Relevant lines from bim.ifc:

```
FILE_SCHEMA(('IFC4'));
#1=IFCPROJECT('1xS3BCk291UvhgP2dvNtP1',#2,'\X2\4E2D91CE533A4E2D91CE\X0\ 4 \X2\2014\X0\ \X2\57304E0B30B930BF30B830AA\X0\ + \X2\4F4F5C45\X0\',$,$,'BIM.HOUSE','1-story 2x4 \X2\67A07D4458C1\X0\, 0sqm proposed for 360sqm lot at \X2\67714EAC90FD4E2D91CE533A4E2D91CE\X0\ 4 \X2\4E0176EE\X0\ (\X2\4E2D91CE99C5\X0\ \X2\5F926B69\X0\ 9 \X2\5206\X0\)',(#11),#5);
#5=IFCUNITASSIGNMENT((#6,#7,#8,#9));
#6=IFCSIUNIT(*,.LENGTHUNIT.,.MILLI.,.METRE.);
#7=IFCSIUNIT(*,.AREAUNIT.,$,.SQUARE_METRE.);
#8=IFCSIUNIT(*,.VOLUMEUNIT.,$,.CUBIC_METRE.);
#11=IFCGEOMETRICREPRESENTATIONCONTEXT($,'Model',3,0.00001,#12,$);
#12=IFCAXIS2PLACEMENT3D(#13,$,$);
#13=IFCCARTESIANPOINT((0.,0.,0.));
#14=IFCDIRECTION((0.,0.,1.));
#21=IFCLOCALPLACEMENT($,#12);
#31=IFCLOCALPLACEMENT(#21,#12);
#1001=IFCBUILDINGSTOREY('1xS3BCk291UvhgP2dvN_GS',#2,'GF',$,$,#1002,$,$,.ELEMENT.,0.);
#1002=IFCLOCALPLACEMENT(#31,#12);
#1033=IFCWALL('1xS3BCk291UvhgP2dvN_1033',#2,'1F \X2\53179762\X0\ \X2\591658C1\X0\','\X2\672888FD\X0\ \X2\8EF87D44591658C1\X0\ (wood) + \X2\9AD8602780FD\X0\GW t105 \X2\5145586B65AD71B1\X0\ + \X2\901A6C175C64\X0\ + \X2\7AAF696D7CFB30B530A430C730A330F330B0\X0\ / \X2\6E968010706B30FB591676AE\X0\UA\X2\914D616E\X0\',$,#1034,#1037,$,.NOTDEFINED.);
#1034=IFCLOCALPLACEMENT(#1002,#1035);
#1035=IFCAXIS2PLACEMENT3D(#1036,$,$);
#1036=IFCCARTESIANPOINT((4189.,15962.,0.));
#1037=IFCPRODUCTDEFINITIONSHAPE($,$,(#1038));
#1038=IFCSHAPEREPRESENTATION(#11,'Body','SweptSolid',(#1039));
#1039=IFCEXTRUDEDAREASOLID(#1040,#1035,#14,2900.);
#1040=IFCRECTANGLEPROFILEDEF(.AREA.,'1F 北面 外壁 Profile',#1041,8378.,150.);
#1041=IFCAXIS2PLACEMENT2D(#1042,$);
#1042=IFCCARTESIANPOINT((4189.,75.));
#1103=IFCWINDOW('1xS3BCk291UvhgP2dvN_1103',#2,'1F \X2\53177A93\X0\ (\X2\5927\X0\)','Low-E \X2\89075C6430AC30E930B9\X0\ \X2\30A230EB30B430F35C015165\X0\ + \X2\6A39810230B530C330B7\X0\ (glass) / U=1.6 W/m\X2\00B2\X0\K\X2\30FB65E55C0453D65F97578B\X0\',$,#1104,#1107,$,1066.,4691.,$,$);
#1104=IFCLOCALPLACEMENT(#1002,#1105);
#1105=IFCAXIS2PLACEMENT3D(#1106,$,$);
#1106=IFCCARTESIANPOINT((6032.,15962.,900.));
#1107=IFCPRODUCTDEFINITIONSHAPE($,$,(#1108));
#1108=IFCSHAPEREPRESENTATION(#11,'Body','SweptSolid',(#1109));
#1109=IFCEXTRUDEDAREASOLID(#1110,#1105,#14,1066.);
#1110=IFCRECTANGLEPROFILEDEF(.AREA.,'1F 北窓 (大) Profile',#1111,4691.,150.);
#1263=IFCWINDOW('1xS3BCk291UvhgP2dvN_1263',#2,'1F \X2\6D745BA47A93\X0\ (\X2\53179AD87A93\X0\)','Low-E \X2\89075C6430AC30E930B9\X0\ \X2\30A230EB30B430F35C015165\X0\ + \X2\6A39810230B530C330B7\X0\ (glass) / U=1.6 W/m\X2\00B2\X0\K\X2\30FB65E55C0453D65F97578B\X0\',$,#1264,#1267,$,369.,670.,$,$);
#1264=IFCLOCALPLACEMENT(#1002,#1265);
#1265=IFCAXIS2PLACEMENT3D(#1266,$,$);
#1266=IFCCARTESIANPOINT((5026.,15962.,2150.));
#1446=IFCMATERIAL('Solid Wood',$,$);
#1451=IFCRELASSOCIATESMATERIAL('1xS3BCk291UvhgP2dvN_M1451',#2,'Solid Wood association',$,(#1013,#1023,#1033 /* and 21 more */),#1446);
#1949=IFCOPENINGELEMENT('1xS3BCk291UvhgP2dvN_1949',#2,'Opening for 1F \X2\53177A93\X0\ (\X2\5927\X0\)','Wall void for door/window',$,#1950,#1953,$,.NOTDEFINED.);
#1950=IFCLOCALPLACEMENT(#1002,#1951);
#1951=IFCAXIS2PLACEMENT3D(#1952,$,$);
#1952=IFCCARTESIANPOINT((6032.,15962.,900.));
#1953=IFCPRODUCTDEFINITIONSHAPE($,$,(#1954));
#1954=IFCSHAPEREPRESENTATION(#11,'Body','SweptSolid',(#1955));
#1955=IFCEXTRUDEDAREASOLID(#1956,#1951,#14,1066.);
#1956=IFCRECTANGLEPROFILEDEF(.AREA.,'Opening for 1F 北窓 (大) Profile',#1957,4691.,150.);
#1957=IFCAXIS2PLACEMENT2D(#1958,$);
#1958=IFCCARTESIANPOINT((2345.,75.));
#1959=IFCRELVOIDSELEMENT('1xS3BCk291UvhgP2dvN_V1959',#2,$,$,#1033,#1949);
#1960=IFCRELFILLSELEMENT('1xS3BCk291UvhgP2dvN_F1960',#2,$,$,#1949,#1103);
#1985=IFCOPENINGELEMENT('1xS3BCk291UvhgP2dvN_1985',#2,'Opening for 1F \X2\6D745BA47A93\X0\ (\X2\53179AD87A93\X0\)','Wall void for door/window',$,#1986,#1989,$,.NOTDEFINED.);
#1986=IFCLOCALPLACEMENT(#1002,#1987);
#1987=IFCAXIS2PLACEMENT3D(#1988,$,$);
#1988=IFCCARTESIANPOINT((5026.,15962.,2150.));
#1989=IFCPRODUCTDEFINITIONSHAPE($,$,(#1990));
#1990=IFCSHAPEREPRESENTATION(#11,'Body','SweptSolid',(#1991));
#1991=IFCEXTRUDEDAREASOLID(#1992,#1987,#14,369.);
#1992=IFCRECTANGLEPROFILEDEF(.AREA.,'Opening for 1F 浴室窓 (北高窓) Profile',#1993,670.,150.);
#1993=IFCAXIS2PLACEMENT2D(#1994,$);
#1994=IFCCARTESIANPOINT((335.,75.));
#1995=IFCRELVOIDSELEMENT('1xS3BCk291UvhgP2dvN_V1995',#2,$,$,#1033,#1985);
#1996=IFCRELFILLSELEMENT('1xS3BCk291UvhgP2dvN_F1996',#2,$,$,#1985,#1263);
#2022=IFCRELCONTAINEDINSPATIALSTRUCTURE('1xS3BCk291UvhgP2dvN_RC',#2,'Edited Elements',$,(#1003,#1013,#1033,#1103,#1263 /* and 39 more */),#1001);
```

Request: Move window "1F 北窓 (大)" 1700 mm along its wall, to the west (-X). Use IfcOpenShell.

```python
import ifcopenshell
import ifcopenshell.api.geometry
import ifcopenshell.util.placement
import ifcopenshell.util.unit

model = ifcopenshell.open("bim.ifc")
unit_scale = ifcopenshell.util.unit.calculate_unit_scale(model)

window = model.by_id(1103)
opening = window.FillsVoids[0].RelatingOpeningElement
wall = opening.VoidsElements[0].RelatingBuildingElement

wall_matrix = ifcopenshell.util.placement.get_local_placement(wall.ObjectPlacement)
shift = wall_matrix[:3, 0] * -1.7 / unit_scale
before = ifcopenshell.util.placement.get_local_placement(window.ObjectPlacement)[:3, 3].copy()

# The window is not placed relative to its opening, so move both.
for product in (opening, window):
    matrix = ifcopenshell.util.placement.get_local_placement(product.ObjectPlacement)
    matrix[:3, 3] += shift
    ifcopenshell.api.geometry.edit_object_placement(model, product=product, matrix=matrix, is_si=False)

after = ifcopenshell.util.placement.get_local_placement(window.ObjectPlacement)[:3, 3]
print("window moved by", (after - before).round(3) + 0.0)

model.write("bim_rev.ifc")
```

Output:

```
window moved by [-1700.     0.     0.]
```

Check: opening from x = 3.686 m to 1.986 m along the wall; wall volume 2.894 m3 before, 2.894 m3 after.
